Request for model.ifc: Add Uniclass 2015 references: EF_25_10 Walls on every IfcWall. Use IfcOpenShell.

First a look at what the model holds.

```python
import ifcopenshell

model = ifcopenshell.open("model.ifc")
print(model.schema)
print("classifications:", [c.Name for c in model.by_type("IfcClassification")])
for ifc_class in ("IfcDoor", "IfcRoof", "IfcStair", "IfcWall", "IfcWindow"):
    print(ifc_class, len(model.by_type(ifc_class)))
```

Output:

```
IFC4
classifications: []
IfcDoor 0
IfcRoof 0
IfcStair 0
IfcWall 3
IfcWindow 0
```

```python
import ifcopenshell
import ifcopenshell.api.classification

model = ifcopenshell.open("model.ifc")

system = ifcopenshell.api.classification.add_classification(model, classification="Uniclass 2015")

codes = {
    "IfcWall": ("EF_25_10", "Walls"),
}
for ifc_class, (code, name) in codes.items():
    products = model.by_type(ifc_class)
    ifcopenshell.api.classification.add_reference(
        model, products=products, classification=system, identification=code, name=name
    )
    print(code, len(products))

model.write("model-out.ifc")
```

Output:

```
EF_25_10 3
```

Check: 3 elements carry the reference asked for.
